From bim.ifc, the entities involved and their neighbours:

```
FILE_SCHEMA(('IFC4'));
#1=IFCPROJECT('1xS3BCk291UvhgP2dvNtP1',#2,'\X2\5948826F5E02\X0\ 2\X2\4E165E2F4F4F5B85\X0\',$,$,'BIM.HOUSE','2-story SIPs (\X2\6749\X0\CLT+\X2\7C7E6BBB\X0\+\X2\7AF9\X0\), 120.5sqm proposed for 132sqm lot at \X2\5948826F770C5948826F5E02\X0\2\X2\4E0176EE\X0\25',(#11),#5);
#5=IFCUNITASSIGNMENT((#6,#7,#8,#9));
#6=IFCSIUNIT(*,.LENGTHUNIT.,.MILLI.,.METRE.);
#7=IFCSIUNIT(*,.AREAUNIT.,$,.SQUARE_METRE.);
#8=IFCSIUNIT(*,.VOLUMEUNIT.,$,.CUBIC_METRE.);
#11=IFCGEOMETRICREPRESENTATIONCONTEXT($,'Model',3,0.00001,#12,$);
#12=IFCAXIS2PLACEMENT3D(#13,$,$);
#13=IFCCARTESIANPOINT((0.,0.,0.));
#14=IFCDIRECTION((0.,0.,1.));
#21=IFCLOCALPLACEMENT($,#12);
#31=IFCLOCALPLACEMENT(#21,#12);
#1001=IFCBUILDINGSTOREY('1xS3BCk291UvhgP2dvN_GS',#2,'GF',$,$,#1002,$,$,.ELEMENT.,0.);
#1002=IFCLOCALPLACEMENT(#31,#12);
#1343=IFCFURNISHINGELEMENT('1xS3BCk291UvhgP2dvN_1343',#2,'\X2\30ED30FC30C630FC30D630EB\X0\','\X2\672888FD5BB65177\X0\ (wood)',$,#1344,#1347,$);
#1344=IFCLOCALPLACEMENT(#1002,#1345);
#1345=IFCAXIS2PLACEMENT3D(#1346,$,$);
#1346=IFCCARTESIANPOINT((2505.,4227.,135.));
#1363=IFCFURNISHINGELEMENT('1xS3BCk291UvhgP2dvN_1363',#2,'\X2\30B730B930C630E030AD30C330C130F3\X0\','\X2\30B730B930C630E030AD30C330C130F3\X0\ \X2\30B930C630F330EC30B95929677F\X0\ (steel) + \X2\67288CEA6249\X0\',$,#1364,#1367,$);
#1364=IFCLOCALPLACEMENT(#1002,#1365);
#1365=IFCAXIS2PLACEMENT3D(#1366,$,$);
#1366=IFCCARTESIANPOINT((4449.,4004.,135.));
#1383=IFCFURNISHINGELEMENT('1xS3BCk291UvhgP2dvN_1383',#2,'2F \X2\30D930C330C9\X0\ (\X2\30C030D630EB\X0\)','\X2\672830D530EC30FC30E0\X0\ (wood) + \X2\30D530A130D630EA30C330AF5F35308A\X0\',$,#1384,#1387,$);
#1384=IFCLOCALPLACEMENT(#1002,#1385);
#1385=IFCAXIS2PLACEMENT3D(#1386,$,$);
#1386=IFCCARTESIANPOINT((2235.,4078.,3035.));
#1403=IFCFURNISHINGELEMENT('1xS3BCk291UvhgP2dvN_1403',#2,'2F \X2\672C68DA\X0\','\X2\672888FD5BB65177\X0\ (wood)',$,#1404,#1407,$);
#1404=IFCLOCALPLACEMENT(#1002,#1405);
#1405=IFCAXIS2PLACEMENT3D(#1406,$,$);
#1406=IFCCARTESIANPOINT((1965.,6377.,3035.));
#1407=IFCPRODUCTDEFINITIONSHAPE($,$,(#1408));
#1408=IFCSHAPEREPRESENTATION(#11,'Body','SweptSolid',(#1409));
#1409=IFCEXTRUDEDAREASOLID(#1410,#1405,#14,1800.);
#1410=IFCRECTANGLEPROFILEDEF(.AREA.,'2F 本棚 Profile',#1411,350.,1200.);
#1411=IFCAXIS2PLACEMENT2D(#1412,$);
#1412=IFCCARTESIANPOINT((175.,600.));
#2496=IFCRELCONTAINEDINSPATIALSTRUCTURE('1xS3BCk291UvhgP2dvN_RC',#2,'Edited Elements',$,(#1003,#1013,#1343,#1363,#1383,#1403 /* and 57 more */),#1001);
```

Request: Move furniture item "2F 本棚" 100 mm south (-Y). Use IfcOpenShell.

```python
import ifcopenshell
import ifcopenshell.api.geometry
import ifcopenshell.util.placement
import ifcopenshell.util.unit

model = ifcopenshell.open("bim.ifc")
unit_scale = ifcopenshell.util.unit.calculate_unit_scale(model)

item = model.by_id(1403)
matrix = ifcopenshell.util.placement.get_local_placement(item.ObjectPlacement)
matrix[1, 3] -= 0.1 / unit_scale
ifcopenshell.api.geometry.edit_object_placement(model, product=item, matrix=matrix, is_si=False)

print(ifcopenshell.util.placement.get_local_placement(item.ObjectPlacement).round(3) + 0.0)

model.write("bim_edited.ifc")
```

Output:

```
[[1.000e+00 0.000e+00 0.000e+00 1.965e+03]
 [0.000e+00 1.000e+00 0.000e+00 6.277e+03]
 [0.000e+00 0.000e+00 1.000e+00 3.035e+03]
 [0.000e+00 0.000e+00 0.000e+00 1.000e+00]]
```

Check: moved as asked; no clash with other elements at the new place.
